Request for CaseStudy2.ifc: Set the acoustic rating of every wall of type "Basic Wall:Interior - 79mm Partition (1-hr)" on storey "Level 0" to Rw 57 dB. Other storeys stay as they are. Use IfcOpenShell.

First a look at what the model holds.

```python
import ifcopenshell
import ifcopenshell.util.element

model = ifcopenshell.open("CaseStudy2.ifc")
print(model.schema)
storey = next(s for s in model.by_type("IfcBuildingStorey") if s.Name == "Level 0")
walls = [e for e in ifcopenshell.util.element.get_decomposition(storey) if e.is_a("IfcWall")]
seen = {}
for e in walls:
    element_type = ifcopenshell.util.element.get_type(e)
    key = (element_type.Name if element_type != e and element_type else None, ifcopenshell.util.element.get_pset(e, "Pset_WallCommon", "AcousticRating"))
    seen[key] = seen.get(key, 0) + 1
for (name, value), count in sorted(seen.items(), key=str):
    print(count, "x", name, "|", value)
```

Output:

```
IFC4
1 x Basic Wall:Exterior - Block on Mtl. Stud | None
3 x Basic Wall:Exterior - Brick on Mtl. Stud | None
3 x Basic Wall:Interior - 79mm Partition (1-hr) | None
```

```python
import ifcopenshell
import ifcopenshell.api.pset
import ifcopenshell.util.element

model = ifcopenshell.open("CaseStudy2.ifc")

storey = next(s for s in model.by_type("IfcBuildingStorey") if s.Name == "Level 0")
walls = [e for e in ifcopenshell.util.element.get_decomposition(storey) if e.is_a("IfcWall")]

count = 0
for e in walls:
    element_type = ifcopenshell.util.element.get_type(e)
    if element_type in (None, e) or element_type.Name != "Basic Wall:Interior - 79mm Partition (1-hr)":
        continue
    # add_pset returns the element's existing set when there is one.
    pset = ifcopenshell.api.pset.add_pset(model, product=e, name="Pset_WallCommon")
    ifcopenshell.api.pset.edit_pset(model, pset=pset, properties={"AcousticRating": "Rw 57 dB"})
    count += 1

print(count, "walls updated")

model.write("CaseStudy2_rev.ifc")
```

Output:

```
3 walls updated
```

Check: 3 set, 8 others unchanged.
